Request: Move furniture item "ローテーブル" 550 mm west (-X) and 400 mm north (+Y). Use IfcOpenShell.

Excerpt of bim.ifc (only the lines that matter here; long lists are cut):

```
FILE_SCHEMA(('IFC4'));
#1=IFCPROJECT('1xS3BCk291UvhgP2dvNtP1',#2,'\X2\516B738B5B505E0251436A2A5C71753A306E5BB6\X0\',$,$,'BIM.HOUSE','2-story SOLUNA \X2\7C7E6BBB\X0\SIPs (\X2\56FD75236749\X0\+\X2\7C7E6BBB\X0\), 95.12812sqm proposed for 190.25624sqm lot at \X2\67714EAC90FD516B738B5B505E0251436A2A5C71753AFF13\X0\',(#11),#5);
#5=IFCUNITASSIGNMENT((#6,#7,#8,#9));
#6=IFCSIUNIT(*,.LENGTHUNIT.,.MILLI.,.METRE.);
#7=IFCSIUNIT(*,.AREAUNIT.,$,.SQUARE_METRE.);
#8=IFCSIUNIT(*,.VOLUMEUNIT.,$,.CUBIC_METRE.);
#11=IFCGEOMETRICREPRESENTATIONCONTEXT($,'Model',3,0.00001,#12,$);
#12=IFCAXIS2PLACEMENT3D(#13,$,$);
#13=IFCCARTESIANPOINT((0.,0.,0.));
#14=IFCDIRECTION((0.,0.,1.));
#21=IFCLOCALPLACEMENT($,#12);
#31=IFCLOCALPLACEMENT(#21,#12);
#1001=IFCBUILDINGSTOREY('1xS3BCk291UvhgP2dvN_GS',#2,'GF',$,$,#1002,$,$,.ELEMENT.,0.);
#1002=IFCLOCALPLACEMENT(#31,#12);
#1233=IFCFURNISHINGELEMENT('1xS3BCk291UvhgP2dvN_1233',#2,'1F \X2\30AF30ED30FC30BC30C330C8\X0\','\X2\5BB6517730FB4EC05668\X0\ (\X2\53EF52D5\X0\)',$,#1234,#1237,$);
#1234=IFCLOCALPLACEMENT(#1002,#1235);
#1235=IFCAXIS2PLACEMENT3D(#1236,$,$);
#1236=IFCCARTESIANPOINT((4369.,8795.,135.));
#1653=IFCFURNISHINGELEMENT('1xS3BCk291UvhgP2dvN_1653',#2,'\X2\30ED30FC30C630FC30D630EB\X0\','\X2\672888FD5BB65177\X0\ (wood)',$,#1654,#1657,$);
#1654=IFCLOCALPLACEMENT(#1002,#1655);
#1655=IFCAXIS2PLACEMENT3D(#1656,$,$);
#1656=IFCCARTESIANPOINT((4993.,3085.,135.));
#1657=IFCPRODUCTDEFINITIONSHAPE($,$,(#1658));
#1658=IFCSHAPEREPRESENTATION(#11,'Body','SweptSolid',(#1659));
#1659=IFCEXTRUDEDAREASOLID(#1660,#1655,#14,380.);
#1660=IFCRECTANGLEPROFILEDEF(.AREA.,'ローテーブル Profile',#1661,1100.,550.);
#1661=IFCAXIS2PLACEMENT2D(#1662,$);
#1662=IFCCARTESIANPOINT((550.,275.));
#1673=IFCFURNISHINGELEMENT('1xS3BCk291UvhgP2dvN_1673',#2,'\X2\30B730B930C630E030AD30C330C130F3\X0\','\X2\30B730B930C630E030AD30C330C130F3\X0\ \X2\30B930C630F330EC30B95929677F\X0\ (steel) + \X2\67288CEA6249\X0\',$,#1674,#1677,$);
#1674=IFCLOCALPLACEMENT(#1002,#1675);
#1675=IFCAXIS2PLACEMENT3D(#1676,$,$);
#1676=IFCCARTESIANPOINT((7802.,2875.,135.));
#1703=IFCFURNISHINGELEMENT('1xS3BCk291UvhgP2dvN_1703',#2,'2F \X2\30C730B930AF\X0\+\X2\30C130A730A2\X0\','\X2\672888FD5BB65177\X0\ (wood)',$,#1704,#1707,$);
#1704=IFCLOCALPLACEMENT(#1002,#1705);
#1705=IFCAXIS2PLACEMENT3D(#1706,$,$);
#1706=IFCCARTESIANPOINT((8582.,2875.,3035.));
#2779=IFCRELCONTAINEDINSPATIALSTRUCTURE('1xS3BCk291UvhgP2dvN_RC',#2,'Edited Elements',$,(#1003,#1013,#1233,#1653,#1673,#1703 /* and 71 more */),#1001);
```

```python
import ifcopenshell
import ifcopenshell.api.geometry
import ifcopenshell.util.placement
import ifcopenshell.util.unit

model = ifcopenshell.open("bim.ifc")
unit_scale = ifcopenshell.util.unit.calculate_unit_scale(model)

item = model.by_id(1653)
matrix = ifcopenshell.util.placement.get_local_placement(item.ObjectPlacement)
matrix[0, 3] -= 0.55 / unit_scale
matrix[1, 3] += 0.4 / unit_scale
ifcopenshell.api.geometry.edit_object_placement(model, product=item, matrix=matrix, is_si=False)

print(ifcopenshell.util.placement.get_local_placement(item.ObjectPlacement).round(3) + 0.0)

model.write("bim-out.ifc")
```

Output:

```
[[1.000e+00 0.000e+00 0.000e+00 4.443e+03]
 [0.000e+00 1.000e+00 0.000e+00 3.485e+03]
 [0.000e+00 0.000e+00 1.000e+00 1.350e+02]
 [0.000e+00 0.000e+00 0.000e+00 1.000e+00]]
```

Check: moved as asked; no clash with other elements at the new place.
